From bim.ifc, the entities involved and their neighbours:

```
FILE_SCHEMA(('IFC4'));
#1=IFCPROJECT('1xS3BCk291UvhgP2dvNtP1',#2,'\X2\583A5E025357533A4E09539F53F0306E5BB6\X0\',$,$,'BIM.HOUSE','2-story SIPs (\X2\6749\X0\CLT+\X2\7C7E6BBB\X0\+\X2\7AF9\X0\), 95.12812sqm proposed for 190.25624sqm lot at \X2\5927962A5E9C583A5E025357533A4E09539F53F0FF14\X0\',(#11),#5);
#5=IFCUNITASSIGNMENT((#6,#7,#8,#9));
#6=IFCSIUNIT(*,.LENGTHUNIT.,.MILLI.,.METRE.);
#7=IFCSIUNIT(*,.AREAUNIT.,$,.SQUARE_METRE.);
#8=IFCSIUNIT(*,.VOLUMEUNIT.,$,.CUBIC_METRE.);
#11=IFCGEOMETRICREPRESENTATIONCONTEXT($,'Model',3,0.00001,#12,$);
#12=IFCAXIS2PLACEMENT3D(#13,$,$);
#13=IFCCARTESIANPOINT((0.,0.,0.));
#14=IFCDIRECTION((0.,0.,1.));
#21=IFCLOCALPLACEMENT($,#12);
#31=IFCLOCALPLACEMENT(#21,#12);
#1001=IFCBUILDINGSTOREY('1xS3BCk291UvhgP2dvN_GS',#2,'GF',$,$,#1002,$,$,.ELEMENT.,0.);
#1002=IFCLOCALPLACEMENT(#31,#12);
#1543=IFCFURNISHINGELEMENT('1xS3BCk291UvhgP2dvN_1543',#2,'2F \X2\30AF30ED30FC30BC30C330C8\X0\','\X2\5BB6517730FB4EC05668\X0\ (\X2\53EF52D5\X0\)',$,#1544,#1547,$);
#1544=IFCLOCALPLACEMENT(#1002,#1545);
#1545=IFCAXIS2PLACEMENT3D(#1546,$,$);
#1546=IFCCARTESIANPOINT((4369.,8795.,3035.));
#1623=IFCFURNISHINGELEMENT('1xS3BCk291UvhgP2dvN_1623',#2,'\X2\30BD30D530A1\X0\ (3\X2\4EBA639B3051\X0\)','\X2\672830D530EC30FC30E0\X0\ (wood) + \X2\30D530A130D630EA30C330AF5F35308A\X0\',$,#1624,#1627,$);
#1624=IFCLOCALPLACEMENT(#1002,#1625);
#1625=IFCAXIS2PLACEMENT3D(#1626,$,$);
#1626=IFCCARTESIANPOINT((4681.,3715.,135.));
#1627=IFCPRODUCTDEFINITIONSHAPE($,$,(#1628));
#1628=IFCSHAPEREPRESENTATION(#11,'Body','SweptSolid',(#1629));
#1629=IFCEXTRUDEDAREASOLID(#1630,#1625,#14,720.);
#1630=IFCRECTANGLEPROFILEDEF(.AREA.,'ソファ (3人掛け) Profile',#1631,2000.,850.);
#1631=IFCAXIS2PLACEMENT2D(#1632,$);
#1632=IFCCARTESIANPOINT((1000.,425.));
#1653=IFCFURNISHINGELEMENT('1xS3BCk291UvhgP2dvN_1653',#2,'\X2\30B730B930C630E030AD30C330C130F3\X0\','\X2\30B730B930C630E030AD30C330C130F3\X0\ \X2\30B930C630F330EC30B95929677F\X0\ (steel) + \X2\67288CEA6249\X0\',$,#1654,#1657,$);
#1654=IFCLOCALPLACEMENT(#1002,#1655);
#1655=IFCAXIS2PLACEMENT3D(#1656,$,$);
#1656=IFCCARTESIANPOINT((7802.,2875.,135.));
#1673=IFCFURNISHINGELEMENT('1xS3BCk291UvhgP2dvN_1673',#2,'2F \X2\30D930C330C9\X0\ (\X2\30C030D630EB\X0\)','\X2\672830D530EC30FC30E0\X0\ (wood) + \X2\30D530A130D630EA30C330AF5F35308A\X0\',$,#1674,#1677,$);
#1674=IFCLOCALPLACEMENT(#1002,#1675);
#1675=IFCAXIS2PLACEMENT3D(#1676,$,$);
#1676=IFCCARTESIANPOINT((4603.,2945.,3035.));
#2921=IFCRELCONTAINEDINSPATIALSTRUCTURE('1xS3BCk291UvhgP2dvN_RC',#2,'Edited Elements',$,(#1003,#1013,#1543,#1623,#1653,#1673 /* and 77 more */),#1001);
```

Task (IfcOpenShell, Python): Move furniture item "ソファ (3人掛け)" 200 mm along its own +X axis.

```python
import ifcopenshell
import ifcopenshell.api.geometry
import ifcopenshell.util.placement
import ifcopenshell.util.unit

model = ifcopenshell.open("bim.ifc")
unit_scale = ifcopenshell.util.unit.calculate_unit_scale(model)

item = model.by_guid("1xS3BCk291UvhgP2dvN_1623")
matrix = ifcopenshell.util.placement.get_local_placement(item.ObjectPlacement)
matrix[:3, 3] += matrix[:3, 0] * 0.2 / unit_scale
ifcopenshell.api.geometry.edit_object_placement(model, product=item, matrix=matrix, is_si=False)

print(ifcopenshell.util.placement.get_local_placement(item.ObjectPlacement).round(3) + 0.0)

model.write("bim_v2.ifc")
```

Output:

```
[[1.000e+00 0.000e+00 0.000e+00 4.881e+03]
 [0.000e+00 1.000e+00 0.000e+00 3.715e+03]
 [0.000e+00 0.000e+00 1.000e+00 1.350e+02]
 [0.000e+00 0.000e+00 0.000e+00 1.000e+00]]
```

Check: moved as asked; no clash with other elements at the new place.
